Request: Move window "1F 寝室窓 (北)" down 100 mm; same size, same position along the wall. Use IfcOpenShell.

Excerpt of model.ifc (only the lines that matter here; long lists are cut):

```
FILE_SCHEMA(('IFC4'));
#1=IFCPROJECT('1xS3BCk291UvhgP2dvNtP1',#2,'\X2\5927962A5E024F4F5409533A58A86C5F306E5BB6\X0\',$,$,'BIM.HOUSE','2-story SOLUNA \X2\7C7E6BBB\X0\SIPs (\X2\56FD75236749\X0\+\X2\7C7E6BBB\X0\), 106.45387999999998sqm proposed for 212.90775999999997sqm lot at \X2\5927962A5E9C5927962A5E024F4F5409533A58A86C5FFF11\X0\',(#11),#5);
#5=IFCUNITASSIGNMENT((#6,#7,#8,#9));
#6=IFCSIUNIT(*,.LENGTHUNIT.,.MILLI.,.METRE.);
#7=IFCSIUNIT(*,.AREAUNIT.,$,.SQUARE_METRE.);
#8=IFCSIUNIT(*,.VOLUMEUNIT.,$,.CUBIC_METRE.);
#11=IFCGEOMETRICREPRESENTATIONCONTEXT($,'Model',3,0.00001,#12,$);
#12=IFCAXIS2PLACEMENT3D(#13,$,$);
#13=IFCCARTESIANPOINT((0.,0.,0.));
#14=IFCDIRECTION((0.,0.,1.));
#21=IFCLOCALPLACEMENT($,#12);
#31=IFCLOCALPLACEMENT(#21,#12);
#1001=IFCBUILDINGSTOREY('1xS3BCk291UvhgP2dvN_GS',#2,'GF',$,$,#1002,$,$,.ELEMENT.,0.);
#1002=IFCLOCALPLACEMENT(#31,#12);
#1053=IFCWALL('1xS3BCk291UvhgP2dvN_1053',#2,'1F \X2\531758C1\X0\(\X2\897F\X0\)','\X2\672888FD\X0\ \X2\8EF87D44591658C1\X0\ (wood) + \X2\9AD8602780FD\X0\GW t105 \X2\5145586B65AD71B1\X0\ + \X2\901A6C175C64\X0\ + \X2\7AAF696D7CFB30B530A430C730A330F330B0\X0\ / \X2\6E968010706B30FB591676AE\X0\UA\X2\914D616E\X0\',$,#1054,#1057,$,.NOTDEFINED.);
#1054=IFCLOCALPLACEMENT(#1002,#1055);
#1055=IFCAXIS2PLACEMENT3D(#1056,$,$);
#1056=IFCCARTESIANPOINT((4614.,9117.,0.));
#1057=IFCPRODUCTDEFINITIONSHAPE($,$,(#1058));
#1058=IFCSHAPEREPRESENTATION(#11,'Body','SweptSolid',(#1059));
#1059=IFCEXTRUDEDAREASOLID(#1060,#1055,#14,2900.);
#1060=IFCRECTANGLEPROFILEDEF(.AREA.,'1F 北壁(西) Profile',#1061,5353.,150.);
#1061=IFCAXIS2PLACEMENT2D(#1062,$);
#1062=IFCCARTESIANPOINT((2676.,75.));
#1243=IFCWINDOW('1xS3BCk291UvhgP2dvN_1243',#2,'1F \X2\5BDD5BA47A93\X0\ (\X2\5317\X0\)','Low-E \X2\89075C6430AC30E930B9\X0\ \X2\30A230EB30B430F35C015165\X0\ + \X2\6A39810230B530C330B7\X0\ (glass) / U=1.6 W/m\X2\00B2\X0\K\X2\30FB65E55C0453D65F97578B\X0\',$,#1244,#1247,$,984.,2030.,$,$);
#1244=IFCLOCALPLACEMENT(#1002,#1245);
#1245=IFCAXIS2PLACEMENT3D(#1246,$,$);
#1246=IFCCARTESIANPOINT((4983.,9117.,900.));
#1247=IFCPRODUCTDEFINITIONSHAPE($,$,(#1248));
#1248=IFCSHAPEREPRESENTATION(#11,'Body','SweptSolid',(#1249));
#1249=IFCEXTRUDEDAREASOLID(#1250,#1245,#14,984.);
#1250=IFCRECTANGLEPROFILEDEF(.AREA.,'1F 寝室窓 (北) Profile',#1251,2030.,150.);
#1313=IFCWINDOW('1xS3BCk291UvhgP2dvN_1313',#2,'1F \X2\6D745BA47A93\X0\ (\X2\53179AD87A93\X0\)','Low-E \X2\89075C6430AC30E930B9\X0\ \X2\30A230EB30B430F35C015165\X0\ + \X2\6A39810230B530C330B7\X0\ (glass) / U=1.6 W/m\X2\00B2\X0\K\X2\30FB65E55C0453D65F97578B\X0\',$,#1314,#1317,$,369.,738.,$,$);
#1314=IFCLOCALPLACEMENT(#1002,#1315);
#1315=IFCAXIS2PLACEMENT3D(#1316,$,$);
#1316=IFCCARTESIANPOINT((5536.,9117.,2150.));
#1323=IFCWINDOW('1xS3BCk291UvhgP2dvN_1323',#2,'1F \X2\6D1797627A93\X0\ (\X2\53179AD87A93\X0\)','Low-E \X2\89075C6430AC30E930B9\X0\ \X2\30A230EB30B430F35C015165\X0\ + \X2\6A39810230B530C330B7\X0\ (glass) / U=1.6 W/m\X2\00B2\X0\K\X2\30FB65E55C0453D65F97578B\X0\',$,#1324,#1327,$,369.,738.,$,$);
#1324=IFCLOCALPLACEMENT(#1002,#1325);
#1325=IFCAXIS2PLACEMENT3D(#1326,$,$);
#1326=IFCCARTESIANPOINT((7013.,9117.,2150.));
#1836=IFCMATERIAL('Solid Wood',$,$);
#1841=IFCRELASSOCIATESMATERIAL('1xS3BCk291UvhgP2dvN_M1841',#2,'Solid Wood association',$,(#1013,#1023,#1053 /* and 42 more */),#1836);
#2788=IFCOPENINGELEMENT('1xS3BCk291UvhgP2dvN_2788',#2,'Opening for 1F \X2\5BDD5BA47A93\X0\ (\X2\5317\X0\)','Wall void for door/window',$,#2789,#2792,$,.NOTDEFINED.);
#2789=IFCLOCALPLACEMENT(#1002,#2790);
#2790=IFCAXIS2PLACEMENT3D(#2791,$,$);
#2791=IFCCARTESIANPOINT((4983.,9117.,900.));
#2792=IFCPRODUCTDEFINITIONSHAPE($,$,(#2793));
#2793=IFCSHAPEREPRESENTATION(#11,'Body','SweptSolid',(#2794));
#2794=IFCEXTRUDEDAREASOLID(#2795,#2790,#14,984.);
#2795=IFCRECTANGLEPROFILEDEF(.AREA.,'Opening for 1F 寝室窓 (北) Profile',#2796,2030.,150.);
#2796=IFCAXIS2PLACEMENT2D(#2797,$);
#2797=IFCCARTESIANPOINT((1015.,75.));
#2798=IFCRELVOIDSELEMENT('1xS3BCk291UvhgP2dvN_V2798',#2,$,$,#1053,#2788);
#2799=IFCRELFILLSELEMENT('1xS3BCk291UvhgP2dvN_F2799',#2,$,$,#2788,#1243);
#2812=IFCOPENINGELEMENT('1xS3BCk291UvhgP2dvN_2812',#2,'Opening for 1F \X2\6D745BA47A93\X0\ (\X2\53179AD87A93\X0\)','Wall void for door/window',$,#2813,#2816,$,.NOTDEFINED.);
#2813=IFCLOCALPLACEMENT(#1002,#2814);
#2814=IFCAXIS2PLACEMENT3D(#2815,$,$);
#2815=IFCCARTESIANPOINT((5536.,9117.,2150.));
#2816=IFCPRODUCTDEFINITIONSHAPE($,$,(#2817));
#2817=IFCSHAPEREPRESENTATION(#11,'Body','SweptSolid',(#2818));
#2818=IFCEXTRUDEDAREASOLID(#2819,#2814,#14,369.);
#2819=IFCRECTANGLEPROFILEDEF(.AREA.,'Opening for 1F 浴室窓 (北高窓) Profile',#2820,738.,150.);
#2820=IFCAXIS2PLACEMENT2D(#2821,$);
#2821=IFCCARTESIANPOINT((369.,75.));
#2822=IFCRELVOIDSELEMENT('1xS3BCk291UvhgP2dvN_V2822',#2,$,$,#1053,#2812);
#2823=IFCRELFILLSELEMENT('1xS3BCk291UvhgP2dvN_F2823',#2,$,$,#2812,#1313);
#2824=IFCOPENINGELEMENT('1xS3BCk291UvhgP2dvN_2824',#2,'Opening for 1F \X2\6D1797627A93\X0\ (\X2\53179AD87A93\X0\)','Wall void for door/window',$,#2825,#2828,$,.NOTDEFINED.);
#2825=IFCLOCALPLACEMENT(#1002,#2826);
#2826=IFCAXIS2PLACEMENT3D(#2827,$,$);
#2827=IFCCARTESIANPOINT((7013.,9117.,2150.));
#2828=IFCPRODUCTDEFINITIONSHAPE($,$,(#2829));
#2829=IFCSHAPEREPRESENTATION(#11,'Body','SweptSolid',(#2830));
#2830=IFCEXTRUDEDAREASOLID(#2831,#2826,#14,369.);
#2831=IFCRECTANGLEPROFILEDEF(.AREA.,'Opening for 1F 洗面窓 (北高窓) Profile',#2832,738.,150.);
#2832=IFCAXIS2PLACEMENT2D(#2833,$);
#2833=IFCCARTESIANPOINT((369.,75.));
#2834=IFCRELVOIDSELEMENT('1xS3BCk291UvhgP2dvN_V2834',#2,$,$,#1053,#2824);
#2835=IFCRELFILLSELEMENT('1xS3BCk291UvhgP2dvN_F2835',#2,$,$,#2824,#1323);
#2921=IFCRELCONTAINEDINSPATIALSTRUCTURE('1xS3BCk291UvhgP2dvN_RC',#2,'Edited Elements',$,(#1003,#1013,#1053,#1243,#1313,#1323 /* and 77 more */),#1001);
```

```python
import numpy as np
import ifcopenshell
import ifcopenshell.api.geometry
import ifcopenshell.util.placement
import ifcopenshell.util.unit

model = ifcopenshell.open("model.ifc")
unit_scale = ifcopenshell.util.unit.calculate_unit_scale(model)

window = model.by_guid("1xS3BCk291UvhgP2dvN_1243")
opening = window.FillsVoids[0].RelatingOpeningElement
dz = -100.0

shift = np.array([0.0, 0.0, dz])
# The window is not placed relative to its opening, so move both.
for product in (opening, window):
    matrix = ifcopenshell.util.placement.get_local_placement(product.ObjectPlacement)
    matrix[:3, 3] += shift
    ifcopenshell.api.geometry.edit_object_placement(model, product=product, matrix=matrix, is_si=False)

print(f"moved by {dz * unit_scale:+.3f} m")

model.write("model-out.ifc")
```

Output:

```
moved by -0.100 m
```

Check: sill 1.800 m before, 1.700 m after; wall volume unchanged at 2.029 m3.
